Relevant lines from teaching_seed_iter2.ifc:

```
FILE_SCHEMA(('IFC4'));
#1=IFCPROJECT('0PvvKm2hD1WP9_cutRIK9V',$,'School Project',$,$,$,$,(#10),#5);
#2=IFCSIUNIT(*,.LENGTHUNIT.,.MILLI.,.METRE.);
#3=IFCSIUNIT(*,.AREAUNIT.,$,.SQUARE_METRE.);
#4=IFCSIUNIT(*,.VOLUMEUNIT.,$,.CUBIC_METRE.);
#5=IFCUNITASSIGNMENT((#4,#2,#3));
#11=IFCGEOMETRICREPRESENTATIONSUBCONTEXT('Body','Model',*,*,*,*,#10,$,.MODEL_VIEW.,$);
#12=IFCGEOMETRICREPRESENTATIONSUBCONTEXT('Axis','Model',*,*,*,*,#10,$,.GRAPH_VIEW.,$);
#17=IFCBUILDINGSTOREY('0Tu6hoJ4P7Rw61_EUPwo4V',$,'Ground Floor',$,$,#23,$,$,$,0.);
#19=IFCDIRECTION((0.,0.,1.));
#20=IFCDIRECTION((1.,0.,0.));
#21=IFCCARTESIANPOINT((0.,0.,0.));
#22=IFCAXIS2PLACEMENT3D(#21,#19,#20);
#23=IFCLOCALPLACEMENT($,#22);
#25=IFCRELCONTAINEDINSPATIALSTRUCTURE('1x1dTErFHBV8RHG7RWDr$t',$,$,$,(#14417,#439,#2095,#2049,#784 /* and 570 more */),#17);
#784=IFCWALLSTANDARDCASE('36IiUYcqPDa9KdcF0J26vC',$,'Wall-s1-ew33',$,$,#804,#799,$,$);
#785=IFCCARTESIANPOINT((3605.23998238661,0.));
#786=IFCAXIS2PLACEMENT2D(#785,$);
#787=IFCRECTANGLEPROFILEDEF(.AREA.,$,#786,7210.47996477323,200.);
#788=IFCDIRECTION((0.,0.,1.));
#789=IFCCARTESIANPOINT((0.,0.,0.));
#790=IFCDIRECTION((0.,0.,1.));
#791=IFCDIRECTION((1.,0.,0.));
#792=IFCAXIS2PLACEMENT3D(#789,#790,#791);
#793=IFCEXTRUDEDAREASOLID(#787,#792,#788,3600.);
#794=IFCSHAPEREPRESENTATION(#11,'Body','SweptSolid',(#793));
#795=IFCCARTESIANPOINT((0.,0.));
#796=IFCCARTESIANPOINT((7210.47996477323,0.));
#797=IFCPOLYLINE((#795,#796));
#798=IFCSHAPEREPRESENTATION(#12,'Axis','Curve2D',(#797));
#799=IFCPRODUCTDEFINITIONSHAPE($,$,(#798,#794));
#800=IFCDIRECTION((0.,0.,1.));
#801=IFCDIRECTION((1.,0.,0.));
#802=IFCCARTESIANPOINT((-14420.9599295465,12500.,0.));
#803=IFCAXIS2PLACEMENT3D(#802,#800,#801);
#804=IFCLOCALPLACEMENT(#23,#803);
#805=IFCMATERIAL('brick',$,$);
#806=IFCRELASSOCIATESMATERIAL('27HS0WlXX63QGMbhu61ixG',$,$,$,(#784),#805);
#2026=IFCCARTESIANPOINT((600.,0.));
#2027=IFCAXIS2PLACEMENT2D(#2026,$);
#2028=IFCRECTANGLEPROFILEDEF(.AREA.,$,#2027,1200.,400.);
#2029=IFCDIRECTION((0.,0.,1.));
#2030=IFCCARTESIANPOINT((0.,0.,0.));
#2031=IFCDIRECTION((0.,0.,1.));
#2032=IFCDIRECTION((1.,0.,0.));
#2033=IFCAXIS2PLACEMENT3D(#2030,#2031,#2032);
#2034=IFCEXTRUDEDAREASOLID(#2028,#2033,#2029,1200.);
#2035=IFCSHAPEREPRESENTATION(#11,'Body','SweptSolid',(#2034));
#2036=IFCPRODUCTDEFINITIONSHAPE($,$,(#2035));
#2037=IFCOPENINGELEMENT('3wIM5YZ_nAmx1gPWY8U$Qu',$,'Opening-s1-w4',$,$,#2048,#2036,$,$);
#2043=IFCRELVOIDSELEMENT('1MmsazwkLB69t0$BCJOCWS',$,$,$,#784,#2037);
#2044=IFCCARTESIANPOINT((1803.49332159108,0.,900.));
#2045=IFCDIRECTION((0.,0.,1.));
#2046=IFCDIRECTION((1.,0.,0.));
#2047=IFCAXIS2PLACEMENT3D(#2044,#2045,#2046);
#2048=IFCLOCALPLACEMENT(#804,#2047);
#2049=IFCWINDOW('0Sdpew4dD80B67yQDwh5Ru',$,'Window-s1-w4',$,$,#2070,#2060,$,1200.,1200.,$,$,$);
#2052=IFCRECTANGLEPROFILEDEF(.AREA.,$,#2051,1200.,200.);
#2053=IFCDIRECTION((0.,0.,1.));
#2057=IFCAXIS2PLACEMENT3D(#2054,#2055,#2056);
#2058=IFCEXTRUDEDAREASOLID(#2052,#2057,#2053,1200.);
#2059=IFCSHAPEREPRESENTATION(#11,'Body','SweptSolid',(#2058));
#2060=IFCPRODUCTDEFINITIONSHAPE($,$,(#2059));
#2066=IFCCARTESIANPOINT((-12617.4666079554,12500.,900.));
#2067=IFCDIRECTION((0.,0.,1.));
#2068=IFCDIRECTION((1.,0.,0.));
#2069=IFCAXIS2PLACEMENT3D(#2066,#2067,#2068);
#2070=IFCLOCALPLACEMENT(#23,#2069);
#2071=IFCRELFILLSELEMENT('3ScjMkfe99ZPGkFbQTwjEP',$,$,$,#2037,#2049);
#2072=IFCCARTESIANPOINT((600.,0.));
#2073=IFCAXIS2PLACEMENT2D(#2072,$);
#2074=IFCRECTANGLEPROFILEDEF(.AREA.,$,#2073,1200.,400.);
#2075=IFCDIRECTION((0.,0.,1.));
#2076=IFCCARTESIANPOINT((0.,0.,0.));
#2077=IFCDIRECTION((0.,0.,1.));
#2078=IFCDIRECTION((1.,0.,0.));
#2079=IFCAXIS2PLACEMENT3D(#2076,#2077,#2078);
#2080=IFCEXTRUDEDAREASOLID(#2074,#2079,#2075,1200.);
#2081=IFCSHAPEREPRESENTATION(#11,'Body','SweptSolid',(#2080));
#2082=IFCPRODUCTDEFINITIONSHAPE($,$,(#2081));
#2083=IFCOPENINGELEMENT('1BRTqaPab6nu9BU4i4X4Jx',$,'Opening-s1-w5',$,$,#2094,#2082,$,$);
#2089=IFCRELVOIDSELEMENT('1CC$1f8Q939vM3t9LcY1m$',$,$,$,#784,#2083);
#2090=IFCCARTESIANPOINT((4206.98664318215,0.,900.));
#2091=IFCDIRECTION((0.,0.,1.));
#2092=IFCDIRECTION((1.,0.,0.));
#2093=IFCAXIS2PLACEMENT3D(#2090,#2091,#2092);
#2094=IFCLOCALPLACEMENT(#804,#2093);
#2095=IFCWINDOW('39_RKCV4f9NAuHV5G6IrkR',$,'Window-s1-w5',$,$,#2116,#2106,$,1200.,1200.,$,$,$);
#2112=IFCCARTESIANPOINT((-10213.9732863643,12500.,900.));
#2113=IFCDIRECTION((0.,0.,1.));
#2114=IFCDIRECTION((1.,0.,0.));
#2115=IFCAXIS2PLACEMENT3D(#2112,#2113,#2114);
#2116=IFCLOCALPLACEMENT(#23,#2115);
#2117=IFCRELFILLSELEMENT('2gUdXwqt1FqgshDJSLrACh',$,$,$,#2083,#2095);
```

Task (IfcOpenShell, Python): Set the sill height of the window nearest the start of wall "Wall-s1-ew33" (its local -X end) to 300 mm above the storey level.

```python
import numpy as np
import ifcopenshell
import ifcopenshell.api.geometry
import ifcopenshell.geom
import ifcopenshell.util.element
import ifcopenshell.util.placement
import ifcopenshell.util.shape
import ifcopenshell.util.unit

model = ifcopenshell.open("teaching_seed_iter2.ifc")
unit_scale = ifcopenshell.util.unit.calculate_unit_scale(model)

window = model.by_guid("0Sdpew4dD80B67yQDwh5Ru")
opening = window.FillsVoids[0].RelatingOpeningElement
storey = ifcopenshell.util.element.get_container(window, ifc_class="IfcBuildingStorey")
level = ifcopenshell.util.placement.get_local_placement(storey.ObjectPlacement)[2, 3]

# The opening's origin need not be at the sill, so measure its lowest point.
shape = ifcopenshell.geom.create_shape(ifcopenshell.geom.settings(), opening)
bottom = ifcopenshell.util.shape.get_shape_bottom_elevation(shape, shape.geometry) / unit_scale
dz = level + 0.3 / unit_scale - bottom

shift = np.array([0.0, 0.0, dz])
# The window is not placed relative to its opening, so move both.
for product in (opening, window):
    matrix = ifcopenshell.util.placement.get_local_placement(product.ObjectPlacement)
    matrix[:3, 3] += shift
    ifcopenshell.api.geometry.edit_object_placement(model, product=product, matrix=matrix, is_si=False)

print(f"moved by {dz * unit_scale:+.3f} m")

model.write("teaching_seed_iter2_rev.ifc")
```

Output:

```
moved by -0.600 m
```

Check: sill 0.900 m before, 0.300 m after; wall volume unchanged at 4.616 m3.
